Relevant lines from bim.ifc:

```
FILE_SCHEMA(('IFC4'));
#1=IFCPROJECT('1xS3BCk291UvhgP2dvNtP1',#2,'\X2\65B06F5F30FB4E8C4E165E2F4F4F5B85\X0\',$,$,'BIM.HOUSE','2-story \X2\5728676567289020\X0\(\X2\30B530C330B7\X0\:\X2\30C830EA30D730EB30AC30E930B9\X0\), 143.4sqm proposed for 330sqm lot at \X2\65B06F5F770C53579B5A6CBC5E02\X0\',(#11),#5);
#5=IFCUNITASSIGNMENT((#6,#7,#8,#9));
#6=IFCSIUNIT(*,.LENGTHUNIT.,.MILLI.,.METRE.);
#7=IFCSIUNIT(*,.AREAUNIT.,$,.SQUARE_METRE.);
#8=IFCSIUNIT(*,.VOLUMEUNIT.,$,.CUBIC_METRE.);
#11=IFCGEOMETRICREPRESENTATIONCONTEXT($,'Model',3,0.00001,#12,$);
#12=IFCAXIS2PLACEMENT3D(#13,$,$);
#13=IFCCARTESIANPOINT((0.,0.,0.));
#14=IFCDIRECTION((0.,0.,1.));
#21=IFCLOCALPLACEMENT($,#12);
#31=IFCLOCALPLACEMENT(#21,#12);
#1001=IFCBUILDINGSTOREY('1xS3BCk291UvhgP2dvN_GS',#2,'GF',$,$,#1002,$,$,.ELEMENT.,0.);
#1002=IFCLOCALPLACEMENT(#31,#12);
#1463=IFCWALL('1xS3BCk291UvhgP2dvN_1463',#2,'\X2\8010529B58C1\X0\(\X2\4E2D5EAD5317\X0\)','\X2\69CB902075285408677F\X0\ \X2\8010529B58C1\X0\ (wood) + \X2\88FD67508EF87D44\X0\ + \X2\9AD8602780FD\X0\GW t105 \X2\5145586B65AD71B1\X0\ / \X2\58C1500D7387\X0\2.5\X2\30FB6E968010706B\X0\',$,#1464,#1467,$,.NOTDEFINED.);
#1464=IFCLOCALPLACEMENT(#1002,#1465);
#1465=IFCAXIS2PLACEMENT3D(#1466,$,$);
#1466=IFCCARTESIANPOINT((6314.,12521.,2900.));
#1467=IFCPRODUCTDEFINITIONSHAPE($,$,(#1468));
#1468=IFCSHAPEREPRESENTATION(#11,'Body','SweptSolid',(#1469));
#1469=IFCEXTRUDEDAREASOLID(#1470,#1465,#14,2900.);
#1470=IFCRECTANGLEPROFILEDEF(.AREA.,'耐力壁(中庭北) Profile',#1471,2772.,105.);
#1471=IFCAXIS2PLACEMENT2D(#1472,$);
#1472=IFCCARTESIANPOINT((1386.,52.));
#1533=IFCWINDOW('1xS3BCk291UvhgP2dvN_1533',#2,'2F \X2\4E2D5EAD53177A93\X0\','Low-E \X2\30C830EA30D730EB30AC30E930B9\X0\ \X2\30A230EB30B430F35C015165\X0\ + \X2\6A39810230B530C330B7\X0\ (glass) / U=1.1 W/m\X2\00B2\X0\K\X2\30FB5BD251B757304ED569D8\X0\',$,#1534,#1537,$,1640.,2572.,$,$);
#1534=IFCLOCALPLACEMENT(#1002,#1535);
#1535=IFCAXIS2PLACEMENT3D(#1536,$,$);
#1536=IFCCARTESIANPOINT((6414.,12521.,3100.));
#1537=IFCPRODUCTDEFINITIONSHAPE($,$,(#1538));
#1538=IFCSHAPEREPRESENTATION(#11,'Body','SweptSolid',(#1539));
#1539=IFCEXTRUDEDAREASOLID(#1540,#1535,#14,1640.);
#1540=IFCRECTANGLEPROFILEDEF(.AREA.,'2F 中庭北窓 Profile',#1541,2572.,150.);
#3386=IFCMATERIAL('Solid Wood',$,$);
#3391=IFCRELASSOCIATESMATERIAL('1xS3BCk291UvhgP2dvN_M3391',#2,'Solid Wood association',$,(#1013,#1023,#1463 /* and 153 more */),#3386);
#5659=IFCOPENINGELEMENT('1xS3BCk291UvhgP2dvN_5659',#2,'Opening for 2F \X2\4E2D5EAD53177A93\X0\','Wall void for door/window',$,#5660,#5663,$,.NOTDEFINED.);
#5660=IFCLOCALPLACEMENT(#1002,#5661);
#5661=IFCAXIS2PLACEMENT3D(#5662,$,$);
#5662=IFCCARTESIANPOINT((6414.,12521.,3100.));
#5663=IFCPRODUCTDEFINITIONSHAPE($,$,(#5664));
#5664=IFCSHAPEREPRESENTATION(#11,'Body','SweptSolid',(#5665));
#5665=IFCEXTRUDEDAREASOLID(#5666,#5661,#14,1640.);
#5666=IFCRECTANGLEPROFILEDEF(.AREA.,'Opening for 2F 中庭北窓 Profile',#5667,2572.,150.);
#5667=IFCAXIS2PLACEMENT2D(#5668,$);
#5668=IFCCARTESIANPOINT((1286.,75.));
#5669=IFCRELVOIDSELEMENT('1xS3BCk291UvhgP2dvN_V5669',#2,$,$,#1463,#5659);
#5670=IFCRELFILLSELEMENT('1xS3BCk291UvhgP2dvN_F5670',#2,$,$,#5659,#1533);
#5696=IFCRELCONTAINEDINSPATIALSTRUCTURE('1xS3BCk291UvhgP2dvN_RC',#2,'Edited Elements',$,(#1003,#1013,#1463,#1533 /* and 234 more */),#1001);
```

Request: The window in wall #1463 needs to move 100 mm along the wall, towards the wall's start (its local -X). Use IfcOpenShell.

```python
import ifcopenshell
import ifcopenshell.api.geometry
import ifcopenshell.util.placement
import ifcopenshell.util.unit

model = ifcopenshell.open("bim.ifc")
unit_scale = ifcopenshell.util.unit.calculate_unit_scale(model)

window = model.by_guid("1xS3BCk291UvhgP2dvN_1533")
opening = window.FillsVoids[0].RelatingOpeningElement
wall = opening.VoidsElements[0].RelatingBuildingElement

wall_matrix = ifcopenshell.util.placement.get_local_placement(wall.ObjectPlacement)
shift = wall_matrix[:3, 0] * -0.1 / unit_scale
before = ifcopenshell.util.placement.get_local_placement(window.ObjectPlacement)[:3, 3].copy()

# The window is not placed relative to its opening, so move both.
for product in (opening, window):
    matrix = ifcopenshell.util.placement.get_local_placement(product.ObjectPlacement)
    matrix[:3, 3] += shift
    ifcopenshell.api.geometry.edit_object_placement(model, product=product, matrix=matrix, is_si=False)

after = ifcopenshell.util.placement.get_local_placement(window.ObjectPlacement)[:3, 3]
print("window moved by", (after - before).round(3) + 0.0)

model.write("bim_rev.ifc")
```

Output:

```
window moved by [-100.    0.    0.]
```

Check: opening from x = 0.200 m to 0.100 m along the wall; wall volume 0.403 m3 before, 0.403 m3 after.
